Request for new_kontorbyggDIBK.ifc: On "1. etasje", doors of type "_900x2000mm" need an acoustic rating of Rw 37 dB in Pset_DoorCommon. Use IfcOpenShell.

First a look at what the model holds.

```python
import ifcopenshell
import ifcopenshell.util.element

model = ifcopenshell.open("new_kontorbyggDIBK.ifc")
print(model.schema)
storey = next(s for s in model.by_type("IfcBuildingStorey") if s.Name == "1. etasje")
doors = [e for e in ifcopenshell.util.element.get_decomposition(storey) if e.is_a("IfcDoor")]
seen = {}
for e in doors:
    element_type = ifcopenshell.util.element.get_type(e)
    key = (element_type.Name if element_type != e and element_type else None, ifcopenshell.util.element.get_pset(e, "Pset_DoorCommon", "AcousticRating"))
    seen[key] = seen.get(key, 0) + 1
for (name, value), count in sorted(seen.items(), key=str):
    print(count, "x", name, "|", value)
```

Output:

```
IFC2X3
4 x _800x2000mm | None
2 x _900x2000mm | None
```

```python
import ifcopenshell
import ifcopenshell.api.pset
import ifcopenshell.util.element

model = ifcopenshell.open("new_kontorbyggDIBK.ifc")

storey = next(s for s in model.by_type("IfcBuildingStorey") if s.Name == "1. etasje")
doors = [e for e in ifcopenshell.util.element.get_decomposition(storey) if e.is_a("IfcDoor")]

count = 0
for e in doors:
    element_type = ifcopenshell.util.element.get_type(e)
    if element_type in (None, e) or element_type.Name != "_900x2000mm":
        continue
    # add_pset returns the element's existing set when there is one.
    pset = ifcopenshell.api.pset.add_pset(model, product=e, name="Pset_DoorCommon")
    ifcopenshell.api.pset.edit_pset(model, pset=pset, properties={"AcousticRating": "Rw 37 dB"})
    count += 1

print(count, "doors updated")

model.write("new_kontorbyggDIBK_updated.ifc")
```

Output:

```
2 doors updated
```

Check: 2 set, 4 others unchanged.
